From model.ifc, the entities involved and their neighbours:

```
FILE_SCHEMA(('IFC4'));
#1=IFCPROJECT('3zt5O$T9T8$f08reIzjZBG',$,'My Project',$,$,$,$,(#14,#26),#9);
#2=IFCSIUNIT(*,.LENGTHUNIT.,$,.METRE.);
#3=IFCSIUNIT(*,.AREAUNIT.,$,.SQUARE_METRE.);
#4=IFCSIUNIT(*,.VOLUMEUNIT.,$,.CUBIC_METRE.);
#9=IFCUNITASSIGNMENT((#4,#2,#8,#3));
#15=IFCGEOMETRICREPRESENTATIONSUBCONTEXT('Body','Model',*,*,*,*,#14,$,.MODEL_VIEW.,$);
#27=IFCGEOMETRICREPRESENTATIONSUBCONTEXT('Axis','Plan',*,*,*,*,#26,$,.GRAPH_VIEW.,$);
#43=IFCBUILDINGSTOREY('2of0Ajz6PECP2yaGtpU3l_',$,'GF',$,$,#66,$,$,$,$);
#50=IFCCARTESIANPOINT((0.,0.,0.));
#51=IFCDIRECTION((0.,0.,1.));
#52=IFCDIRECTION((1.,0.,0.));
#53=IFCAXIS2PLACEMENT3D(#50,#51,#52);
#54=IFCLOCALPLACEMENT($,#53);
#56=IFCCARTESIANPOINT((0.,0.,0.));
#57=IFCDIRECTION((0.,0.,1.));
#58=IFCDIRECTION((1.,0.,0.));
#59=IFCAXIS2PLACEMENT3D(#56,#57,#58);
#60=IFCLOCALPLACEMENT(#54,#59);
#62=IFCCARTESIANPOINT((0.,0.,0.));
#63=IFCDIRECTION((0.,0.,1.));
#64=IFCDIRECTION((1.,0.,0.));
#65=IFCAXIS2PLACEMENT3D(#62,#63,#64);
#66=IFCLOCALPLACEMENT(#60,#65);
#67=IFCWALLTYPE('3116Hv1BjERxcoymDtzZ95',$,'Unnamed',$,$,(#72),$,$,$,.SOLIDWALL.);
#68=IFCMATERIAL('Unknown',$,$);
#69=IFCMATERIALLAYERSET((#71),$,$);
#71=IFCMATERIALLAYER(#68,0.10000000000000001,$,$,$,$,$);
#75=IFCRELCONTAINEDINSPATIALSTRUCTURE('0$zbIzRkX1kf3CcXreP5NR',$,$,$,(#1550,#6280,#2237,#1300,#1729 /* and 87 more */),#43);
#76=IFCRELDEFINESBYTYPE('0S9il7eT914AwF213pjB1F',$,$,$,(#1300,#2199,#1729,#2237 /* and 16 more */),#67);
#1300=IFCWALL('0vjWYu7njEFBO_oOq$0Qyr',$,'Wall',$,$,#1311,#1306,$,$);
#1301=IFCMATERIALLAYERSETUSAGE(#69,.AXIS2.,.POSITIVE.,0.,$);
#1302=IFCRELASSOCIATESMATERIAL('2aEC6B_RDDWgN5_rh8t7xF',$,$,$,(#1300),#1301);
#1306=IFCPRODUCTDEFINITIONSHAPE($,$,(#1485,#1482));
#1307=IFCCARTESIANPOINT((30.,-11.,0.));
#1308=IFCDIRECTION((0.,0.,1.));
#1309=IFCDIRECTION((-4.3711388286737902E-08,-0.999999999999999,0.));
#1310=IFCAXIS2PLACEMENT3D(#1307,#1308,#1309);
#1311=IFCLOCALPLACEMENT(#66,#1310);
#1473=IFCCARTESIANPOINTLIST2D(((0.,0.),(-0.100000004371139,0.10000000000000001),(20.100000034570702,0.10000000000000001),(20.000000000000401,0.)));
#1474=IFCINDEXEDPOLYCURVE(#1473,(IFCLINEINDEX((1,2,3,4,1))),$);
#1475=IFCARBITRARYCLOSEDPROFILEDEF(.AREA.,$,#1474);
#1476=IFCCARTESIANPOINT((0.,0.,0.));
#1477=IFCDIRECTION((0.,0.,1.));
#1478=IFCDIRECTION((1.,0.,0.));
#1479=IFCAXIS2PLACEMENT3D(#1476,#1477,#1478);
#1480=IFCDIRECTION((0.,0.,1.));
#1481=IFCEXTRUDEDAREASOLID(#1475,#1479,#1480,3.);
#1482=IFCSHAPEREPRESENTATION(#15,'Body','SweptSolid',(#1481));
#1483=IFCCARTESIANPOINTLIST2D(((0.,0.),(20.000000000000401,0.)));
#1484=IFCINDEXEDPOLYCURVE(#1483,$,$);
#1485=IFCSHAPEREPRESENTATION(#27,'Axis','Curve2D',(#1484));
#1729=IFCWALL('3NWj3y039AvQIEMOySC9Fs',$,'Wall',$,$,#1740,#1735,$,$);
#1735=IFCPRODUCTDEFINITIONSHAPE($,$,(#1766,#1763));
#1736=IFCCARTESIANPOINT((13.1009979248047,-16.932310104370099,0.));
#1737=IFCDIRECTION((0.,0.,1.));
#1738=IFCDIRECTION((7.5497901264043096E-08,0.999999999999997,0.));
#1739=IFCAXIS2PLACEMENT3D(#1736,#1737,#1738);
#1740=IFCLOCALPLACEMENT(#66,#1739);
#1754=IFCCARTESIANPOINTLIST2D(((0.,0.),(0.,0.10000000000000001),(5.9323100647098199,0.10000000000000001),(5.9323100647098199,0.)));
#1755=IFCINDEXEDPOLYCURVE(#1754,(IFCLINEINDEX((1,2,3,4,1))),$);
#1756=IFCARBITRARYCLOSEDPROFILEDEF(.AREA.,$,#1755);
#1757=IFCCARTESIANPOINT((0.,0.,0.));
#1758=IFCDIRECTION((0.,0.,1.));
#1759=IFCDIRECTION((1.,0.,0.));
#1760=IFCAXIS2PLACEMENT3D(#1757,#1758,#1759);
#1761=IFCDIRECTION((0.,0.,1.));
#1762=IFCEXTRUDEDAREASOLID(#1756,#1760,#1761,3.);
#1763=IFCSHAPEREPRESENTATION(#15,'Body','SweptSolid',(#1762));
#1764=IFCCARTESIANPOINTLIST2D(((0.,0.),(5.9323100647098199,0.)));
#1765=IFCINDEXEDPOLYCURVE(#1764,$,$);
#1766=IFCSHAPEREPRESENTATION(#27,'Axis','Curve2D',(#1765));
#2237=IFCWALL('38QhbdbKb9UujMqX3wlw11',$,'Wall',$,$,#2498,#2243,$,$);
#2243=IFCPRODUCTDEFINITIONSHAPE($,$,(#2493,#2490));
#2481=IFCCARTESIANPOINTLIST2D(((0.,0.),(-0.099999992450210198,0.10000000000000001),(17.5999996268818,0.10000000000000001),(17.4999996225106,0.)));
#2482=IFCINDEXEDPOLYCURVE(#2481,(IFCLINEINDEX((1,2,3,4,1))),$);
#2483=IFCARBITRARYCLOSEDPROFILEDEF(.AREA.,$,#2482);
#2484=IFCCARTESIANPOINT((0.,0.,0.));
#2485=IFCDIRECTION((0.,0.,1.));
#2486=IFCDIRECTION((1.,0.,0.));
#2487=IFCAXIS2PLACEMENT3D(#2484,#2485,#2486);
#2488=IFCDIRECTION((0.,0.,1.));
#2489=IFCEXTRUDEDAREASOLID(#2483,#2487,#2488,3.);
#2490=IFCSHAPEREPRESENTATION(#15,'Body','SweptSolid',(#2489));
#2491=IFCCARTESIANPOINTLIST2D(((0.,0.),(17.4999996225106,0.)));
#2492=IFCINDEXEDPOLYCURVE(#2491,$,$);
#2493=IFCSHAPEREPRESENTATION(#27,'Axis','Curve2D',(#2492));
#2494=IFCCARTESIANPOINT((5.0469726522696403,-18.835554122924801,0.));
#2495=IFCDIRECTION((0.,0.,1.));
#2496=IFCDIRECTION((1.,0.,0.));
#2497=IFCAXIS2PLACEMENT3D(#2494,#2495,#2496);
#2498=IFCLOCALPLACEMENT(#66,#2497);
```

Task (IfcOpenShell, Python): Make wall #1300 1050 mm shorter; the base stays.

```python
import ifcopenshell
import ifcopenshell.geom
import ifcopenshell.util.representation
import ifcopenshell.util.shape

model = ifcopenshell.open("model.ifc")
settings = ifcopenshell.geom.settings()


def volume(element):
    """Net volume in cubic metres, openings subtracted."""
    shape = ifcopenshell.geom.create_shape(settings, element)
    return ifcopenshell.util.shape.get_volume(shape.geometry)


wall = model.by_id(1300)
before = volume(wall)

body = ifcopenshell.util.representation.get_representation(wall, "Model", "Body")
solid = body.Items[0]
old_height = solid.Depth
solid.Depth -= 1.05
after = volume(wall)

print(f"height {old_height:g} -> {solid.Depth:g}, volume {before:.3f} -> {after:.3f} m3")

model.write("model_rev.ifc")
```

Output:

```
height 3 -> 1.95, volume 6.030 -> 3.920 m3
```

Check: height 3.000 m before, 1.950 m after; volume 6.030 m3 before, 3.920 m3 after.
